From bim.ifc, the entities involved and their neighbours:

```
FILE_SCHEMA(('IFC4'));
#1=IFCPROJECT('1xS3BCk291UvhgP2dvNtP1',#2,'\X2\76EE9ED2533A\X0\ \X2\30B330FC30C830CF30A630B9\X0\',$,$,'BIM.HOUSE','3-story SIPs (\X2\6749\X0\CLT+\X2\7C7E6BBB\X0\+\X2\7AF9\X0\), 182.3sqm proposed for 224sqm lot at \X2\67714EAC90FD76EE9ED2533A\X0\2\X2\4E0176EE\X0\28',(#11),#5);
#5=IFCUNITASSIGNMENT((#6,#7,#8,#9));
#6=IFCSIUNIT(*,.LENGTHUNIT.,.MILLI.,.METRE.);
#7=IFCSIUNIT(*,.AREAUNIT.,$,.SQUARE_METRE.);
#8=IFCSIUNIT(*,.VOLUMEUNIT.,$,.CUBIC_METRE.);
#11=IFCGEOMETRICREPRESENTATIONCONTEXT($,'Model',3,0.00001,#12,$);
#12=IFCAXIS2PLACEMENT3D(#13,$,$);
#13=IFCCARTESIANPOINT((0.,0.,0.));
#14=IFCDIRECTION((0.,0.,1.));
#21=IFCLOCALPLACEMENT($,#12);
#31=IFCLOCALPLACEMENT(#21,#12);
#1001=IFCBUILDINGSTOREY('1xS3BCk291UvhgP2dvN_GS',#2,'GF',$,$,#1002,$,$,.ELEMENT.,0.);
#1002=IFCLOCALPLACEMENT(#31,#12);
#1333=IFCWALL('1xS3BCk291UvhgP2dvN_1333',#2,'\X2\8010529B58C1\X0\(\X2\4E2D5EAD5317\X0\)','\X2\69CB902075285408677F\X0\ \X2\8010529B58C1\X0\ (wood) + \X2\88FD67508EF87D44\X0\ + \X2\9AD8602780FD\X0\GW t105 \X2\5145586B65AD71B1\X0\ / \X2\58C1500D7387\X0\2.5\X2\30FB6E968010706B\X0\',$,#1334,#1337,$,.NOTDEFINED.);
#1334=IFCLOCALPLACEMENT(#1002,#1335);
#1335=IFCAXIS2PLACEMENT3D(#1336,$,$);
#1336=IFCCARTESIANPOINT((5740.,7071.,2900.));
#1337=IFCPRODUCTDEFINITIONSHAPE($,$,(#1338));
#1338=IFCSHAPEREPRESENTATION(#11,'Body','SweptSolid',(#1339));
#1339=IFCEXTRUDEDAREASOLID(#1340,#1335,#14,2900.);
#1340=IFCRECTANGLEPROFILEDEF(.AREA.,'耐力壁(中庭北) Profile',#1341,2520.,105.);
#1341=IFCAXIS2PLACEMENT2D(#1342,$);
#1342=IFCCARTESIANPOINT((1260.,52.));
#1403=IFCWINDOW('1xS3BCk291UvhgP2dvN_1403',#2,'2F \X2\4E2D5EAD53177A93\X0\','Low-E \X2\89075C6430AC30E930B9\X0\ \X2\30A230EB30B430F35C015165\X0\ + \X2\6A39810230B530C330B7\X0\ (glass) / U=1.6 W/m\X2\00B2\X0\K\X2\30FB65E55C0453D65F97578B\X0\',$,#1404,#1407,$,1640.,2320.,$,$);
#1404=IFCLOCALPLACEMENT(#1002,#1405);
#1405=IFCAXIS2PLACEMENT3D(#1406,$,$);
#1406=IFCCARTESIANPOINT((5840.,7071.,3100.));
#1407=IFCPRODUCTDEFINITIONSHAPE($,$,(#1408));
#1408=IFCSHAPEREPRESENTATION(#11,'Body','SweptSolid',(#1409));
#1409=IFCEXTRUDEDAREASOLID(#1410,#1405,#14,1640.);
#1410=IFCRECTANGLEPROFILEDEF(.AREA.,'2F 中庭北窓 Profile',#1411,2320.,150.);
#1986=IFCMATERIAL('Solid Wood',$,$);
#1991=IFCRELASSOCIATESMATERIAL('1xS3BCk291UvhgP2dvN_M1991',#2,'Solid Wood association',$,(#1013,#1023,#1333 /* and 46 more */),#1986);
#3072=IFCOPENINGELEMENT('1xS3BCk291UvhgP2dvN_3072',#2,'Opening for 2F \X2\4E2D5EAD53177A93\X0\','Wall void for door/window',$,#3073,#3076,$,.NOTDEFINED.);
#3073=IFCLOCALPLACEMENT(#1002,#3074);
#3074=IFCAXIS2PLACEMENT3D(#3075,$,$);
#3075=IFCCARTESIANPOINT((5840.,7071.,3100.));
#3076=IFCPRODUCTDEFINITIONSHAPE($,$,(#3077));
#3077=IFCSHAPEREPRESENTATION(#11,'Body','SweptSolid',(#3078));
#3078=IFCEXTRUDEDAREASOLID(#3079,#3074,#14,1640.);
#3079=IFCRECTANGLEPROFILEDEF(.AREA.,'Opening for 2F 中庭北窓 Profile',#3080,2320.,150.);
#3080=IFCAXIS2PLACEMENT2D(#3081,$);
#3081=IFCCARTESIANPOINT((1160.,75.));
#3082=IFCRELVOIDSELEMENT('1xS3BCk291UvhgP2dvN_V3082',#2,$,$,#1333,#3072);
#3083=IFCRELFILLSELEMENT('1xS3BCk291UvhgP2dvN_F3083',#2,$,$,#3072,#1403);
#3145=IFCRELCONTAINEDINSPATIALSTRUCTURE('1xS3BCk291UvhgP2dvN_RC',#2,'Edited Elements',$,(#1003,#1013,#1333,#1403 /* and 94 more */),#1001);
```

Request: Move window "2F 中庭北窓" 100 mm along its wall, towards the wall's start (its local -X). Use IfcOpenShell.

```python
import ifcopenshell
import ifcopenshell.api.geometry
import ifcopenshell.util.placement

model = ifcopenshell.open("bim.ifc")

window = model.by_guid("1xS3BCk291UvhgP2dvN_1403")
opening = window.FillsVoids[0].RelatingOpeningElement
wall = opening.VoidsElements[0].RelatingBuildingElement

wall_matrix = ifcopenshell.util.placement.get_local_placement(wall.ObjectPlacement)
shift = wall_matrix[:3, 0] * -100.0
before = ifcopenshell.util.placement.get_local_placement(window.ObjectPlacement)[:3, 3].copy()

# The window is not placed relative to its opening, so move both.
for product in (opening, window):
    matrix = ifcopenshell.util.placement.get_local_placement(product.ObjectPlacement)
    matrix[:3, 3] += shift
    ifcopenshell.api.geometry.edit_object_placement(model, product=product, matrix=matrix, is_si=False)

after = ifcopenshell.util.placement.get_local_placement(window.ObjectPlacement)[:3, 3]
print("window moved by", (after - before).round(3) + 0.0)

model.write("bim_updated.ifc")
```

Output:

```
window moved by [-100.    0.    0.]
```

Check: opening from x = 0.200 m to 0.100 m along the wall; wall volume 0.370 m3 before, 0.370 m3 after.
